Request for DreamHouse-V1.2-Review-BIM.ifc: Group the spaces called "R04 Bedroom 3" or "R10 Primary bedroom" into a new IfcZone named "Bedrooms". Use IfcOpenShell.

First a look at what the model holds.

```python
import ifcopenshell

model = ifcopenshell.open("DreamHouse-V1.2-Review-BIM.ifc")
print(model.schema)
seen = {}
for space in model.by_type("IfcSpace"):
    seen[space.LongName] = seen.get(space.LongName, 0) + 1
for name, count in sorted(seen.items(), key=str):
    print(count, "x", name)
print("zones:", [z.Name for z in model.by_type("IfcZone")][:20])
```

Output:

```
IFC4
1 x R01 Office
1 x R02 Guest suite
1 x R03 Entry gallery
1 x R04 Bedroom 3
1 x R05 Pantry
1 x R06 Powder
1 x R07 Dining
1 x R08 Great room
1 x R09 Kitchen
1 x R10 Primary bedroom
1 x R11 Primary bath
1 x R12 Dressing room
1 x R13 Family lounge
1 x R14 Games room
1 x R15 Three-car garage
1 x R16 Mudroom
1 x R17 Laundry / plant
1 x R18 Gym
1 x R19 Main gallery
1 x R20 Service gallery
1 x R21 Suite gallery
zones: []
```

```python
import ifcopenshell
import ifcopenshell.api.group
import ifcopenshell.api.root

model = ifcopenshell.open("DreamHouse-V1.2-Review-BIM.ifc")

names = {"R04 Bedroom 3", "R10 Primary bedroom"}
spaces = [s for s in model.by_type("IfcSpace") if s.LongName in names]

zone = ifcopenshell.api.root.create_entity(model, ifc_class="IfcZone", name="Bedrooms")
ifcopenshell.api.group.assign_group(model, products=spaces, group=zone)
print(len(spaces), "spaces in", zone.Name)

model.write("DreamHouse-V1.2-Review-BIM_edited.ifc")
```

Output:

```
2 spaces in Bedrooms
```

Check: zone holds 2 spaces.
